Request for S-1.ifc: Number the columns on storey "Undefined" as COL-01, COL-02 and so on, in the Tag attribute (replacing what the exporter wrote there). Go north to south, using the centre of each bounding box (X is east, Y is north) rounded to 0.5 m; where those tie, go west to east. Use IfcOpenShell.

First a look at what the model holds.

```python
import ifcopenshell
import ifcopenshell.util.element
import ifcopenshell.util.placement

model = ifcopenshell.open("S-1.ifc")
print(model.schema)
storey = next(s for s in model.by_type("IfcBuildingStorey") if s.Name == "Undefined")
columns = [e for e in ifcopenshell.util.element.get_decomposition(storey) if e.is_a("IfcColumn")]
for e in sorted(columns, key=lambda e: e.id()):
    origin = ifcopenshell.util.placement.get_local_placement(e.ObjectPlacement)[:3, 3]
    print(e.id(), e.Tag, e.Name, origin.round(2) + 0.0, sep=" | ")
```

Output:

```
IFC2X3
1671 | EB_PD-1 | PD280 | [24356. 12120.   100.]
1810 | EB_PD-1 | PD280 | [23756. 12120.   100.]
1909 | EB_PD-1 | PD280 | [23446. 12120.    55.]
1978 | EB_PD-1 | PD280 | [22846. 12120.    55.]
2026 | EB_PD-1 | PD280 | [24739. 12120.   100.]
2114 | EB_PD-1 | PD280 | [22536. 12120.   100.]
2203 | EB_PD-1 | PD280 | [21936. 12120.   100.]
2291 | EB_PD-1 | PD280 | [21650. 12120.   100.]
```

```python
import ifcopenshell
import ifcopenshell.geom
import ifcopenshell.util.element
import ifcopenshell.util.shape

model = ifcopenshell.open("S-1.ifc")
settings = ifcopenshell.geom.settings()
settings.set("use-world-coords", True)


def centre(element):
    shape = ifcopenshell.geom.create_shape(settings, element)
    return ifcopenshell.util.shape.get_bbox_centroid(shape.geometry)


storey = next(s for s in model.by_type("IfcBuildingStorey") if s.Name == "Undefined")
columns = [e for e in ifcopenshell.util.element.get_decomposition(storey) if e.is_a("IfcColumn")]

# Insertion points can sit at a corner or the storey origin, so sort by the geometry (in metres).
centres = {e: centre(e) for e in columns}
columns.sort(key=lambda e: (-round(centres[e][1] / 0.5), centres[e][0]))

for i, e in enumerate(columns, start=1):
    number = f"COL-{i:02d}"
    e.Tag = number
    print(e.id(), number)

model.write("S-1_v2.ifc")
```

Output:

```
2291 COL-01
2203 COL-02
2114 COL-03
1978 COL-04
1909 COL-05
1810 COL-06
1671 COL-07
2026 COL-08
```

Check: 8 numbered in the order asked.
